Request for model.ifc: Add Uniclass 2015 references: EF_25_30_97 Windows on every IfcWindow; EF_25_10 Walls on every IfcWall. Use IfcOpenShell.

First a look at what the model holds.

```python
import ifcopenshell

model = ifcopenshell.open("model.ifc")
print(model.schema)
print("classifications:", [c.Name for c in model.by_type("IfcClassification")])
for ifc_class in ("IfcDoor", "IfcRoof", "IfcStair", "IfcWall", "IfcWindow"):
    print(ifc_class, len(model.by_type(ifc_class)))
```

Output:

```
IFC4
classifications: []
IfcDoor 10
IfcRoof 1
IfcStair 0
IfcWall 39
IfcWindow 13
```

```python
import ifcopenshell
import ifcopenshell.api.classification

model = ifcopenshell.open("model.ifc")

system = ifcopenshell.api.classification.add_classification(model, classification="Uniclass 2015")

codes = {
    "IfcWindow": ("EF_25_30_97", "Windows"),
    "IfcWall": ("EF_25_10", "Walls"),
}
for ifc_class, (code, name) in codes.items():
    products = model.by_type(ifc_class)
    ifcopenshell.api.classification.add_reference(
        model, products=products, classification=system, identification=code, name=name
    )
    print(code, len(products))

model.write("model_rev.ifc")
```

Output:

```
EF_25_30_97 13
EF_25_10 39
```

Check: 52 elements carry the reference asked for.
